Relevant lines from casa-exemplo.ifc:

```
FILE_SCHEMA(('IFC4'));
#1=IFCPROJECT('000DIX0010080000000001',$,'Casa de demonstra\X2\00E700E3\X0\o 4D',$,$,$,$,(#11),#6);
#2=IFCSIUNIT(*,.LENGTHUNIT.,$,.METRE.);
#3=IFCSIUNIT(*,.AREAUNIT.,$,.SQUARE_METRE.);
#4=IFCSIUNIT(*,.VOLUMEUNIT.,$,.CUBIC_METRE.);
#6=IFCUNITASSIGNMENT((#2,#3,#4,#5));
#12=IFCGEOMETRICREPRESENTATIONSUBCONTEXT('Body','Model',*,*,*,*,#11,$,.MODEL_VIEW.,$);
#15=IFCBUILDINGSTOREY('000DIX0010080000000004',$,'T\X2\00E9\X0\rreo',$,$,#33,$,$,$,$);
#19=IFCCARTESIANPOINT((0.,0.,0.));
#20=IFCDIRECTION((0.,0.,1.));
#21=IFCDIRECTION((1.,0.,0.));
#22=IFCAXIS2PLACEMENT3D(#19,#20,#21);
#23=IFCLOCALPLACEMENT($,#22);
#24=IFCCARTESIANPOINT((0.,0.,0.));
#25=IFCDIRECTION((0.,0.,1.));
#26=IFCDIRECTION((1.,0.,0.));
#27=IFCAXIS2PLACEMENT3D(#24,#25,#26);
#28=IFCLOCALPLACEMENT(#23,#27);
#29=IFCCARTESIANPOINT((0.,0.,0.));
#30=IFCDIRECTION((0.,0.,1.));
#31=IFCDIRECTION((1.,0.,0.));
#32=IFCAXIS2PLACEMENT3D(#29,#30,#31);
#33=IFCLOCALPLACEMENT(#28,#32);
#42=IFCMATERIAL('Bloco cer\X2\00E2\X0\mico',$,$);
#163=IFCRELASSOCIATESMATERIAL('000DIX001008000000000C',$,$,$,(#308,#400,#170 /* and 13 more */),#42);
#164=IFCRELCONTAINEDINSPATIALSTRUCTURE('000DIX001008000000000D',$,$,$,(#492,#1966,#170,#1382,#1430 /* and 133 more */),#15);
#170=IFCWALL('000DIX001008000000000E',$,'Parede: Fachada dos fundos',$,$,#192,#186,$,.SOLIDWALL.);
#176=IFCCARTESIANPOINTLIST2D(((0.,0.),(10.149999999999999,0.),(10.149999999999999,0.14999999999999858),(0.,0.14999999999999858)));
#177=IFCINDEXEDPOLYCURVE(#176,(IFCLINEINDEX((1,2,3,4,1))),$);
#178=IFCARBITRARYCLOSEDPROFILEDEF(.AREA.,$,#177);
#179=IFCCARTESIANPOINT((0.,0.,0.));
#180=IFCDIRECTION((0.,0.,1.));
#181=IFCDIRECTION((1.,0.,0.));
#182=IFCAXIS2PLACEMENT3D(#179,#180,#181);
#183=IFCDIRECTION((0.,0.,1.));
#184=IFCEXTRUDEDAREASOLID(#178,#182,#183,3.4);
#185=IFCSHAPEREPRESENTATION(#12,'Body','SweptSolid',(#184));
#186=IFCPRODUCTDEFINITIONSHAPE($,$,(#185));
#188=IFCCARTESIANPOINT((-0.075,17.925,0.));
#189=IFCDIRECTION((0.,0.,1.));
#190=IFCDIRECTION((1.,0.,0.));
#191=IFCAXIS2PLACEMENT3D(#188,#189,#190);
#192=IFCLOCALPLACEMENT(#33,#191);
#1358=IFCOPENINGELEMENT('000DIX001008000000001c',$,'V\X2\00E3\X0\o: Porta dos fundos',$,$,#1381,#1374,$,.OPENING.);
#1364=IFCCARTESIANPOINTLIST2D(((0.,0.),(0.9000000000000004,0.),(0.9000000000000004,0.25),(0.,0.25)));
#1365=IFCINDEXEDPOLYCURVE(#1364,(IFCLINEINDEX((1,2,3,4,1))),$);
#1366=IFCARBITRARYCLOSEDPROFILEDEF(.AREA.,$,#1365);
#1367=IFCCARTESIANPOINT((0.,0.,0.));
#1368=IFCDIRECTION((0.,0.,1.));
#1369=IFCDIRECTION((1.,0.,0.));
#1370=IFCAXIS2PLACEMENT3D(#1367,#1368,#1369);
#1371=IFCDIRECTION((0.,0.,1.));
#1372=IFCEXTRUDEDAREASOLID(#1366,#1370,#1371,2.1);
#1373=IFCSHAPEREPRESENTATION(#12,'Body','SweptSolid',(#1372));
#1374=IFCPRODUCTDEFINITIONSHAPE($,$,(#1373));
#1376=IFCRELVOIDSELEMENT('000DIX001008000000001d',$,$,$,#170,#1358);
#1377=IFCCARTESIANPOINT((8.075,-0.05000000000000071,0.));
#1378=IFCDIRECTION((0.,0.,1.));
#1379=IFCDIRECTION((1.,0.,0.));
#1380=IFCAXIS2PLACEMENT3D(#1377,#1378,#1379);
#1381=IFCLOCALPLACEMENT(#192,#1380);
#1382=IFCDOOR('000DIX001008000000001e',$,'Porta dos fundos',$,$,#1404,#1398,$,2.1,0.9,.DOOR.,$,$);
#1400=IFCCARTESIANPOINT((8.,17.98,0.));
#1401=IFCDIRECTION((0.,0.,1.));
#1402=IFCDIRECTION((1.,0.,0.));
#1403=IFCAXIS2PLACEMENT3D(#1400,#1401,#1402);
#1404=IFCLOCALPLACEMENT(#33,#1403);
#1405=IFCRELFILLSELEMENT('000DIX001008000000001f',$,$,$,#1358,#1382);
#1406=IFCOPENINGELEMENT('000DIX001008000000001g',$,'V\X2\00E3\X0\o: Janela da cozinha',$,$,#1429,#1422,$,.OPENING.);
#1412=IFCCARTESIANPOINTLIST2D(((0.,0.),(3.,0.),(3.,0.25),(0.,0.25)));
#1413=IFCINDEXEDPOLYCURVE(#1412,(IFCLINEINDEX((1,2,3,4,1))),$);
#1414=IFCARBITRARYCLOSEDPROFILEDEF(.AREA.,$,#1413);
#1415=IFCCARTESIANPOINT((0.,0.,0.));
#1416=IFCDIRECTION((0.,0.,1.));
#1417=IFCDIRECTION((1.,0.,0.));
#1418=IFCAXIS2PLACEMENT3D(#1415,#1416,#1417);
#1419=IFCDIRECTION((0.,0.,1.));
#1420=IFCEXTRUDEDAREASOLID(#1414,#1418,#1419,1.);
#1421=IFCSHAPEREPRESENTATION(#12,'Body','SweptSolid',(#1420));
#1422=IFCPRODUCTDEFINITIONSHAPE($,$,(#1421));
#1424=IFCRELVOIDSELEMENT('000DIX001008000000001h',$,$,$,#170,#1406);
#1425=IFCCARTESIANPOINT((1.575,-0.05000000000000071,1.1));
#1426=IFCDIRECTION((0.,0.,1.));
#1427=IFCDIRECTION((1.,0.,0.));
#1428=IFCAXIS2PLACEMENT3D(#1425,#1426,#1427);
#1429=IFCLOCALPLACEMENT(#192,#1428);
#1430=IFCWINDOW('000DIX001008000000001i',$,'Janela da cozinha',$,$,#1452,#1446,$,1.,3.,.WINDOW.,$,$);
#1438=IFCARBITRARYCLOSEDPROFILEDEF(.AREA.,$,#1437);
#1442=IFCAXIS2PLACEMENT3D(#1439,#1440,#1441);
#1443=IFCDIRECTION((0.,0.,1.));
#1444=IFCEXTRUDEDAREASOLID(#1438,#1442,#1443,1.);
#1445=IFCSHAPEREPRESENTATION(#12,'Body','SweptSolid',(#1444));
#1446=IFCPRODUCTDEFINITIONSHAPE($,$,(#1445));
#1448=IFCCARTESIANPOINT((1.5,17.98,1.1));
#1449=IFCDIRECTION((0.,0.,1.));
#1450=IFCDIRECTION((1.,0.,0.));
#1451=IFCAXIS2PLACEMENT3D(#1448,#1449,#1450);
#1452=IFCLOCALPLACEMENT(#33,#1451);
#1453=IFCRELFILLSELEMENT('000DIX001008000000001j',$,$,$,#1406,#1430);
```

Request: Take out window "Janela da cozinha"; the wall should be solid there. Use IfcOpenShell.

```python
import ifcopenshell
import ifcopenshell.api.feature
import ifcopenshell.api.root
import ifcopenshell.geom
import ifcopenshell.util.shape

model = ifcopenshell.open("casa-exemplo.ifc")
settings = ifcopenshell.geom.settings()


def volume(element):
    """Net volume in cubic metres, openings subtracted."""
    shape = ifcopenshell.geom.create_shape(settings, element)
    return ifcopenshell.util.shape.get_volume(shape.geometry)


window = model.by_guid("000DIX001008000000001i")
opening = window.FillsVoids[0].RelatingOpeningElement
wall = opening.VoidsElements[0].RelatingBuildingElement
before = volume(wall)

ifcopenshell.api.root.remove_product(model, product=window)
ifcopenshell.api.feature.remove_feature(model, feature=opening)

after = volume(wall)

print(f"wall volume {before:.3f} -> {after:.3f} m3")

model.write("casa-exemplo-out.ifc")
```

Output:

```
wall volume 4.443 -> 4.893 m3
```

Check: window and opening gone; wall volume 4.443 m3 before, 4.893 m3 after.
